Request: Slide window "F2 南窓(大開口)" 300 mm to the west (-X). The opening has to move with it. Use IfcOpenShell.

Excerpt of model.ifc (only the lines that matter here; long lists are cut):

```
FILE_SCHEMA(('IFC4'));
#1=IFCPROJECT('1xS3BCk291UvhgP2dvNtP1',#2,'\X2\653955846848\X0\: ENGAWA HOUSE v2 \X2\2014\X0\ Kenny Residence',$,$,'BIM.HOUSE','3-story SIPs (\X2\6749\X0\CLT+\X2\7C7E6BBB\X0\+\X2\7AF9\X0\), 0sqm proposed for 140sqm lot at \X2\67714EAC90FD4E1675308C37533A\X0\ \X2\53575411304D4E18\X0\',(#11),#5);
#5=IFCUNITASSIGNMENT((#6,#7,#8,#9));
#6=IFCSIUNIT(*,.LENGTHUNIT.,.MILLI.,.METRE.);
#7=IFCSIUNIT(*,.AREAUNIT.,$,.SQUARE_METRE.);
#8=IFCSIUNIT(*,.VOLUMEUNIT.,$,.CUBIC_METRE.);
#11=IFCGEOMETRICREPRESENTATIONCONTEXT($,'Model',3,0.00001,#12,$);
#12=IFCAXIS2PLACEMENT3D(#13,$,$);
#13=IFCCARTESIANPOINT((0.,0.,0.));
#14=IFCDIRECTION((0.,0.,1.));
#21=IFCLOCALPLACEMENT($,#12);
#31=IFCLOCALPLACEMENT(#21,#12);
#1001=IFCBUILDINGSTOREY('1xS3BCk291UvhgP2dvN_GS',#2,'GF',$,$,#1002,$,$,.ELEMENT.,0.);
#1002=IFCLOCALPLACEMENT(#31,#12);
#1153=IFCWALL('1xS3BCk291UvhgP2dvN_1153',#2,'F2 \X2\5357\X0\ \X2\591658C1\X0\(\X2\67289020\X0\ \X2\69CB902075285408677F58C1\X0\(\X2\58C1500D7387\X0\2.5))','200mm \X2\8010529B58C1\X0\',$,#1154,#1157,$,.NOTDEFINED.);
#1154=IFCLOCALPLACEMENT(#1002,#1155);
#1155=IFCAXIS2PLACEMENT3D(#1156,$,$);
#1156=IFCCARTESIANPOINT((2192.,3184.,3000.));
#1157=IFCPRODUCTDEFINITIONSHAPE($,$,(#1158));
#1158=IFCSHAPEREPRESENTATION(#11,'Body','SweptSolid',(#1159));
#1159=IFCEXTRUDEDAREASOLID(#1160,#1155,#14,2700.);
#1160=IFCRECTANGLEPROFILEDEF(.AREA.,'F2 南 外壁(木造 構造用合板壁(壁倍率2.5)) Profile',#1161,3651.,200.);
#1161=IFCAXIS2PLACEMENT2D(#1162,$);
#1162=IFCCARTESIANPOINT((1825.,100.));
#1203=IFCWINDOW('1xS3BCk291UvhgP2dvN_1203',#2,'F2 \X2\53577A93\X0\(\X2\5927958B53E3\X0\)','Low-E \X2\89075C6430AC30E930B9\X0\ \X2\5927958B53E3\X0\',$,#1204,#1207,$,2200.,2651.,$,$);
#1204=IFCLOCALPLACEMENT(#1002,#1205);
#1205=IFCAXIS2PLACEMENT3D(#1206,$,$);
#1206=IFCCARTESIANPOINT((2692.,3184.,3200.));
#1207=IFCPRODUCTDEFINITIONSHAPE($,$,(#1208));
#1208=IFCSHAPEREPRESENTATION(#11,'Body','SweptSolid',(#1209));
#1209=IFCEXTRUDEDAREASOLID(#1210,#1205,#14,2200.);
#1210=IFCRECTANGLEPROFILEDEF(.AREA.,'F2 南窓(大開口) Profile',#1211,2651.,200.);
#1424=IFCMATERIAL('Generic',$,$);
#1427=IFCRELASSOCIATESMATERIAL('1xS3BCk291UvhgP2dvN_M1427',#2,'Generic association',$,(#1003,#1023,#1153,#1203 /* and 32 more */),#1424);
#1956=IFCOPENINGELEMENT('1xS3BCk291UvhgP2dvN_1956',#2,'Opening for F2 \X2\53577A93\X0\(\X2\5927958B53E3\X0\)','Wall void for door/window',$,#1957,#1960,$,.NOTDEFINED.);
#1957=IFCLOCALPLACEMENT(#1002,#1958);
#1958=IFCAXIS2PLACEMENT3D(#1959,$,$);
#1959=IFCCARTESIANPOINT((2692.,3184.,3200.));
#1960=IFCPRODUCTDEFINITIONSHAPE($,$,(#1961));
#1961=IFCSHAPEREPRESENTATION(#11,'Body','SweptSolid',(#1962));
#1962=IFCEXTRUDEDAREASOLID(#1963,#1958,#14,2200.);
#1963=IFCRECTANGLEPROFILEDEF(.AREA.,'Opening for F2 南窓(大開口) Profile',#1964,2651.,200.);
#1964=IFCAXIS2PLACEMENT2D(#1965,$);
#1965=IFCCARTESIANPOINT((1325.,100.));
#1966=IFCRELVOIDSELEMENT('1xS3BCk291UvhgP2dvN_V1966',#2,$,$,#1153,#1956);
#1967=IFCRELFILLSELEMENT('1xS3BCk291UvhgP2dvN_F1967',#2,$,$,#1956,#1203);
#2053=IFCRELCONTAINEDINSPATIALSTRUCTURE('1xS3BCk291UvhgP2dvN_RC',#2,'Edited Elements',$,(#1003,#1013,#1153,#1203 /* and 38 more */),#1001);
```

```python
import ifcopenshell
import ifcopenshell.api.geometry
import ifcopenshell.util.placement

model = ifcopenshell.open("model.ifc")

window = model.by_guid("1xS3BCk291UvhgP2dvN_1203")
opening = window.FillsVoids[0].RelatingOpeningElement
wall = opening.VoidsElements[0].RelatingBuildingElement

wall_matrix = ifcopenshell.util.placement.get_local_placement(wall.ObjectPlacement)
shift = wall_matrix[:3, 0] * -300.0
before = ifcopenshell.util.placement.get_local_placement(window.ObjectPlacement)[:3, 3].copy()

# The window is not placed relative to its opening, so move both.
for product in (opening, window):
    matrix = ifcopenshell.util.placement.get_local_placement(product.ObjectPlacement)
    matrix[:3, 3] += shift
    ifcopenshell.api.geometry.edit_object_placement(model, product=product, matrix=matrix, is_si=False)

after = ifcopenshell.util.placement.get_local_placement(window.ObjectPlacement)[:3, 3]
print("window moved by", (after - before).round(3) + 0.0)

model.write("model_v2.ifc")
```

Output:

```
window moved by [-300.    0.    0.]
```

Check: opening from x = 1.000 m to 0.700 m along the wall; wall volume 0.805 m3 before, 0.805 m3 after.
